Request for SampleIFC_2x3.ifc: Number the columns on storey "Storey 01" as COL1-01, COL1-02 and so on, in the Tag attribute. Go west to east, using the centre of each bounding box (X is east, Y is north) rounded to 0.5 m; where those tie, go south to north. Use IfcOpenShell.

First a look at what the model holds.

```python
import ifcopenshell
import ifcopenshell.util.element
import ifcopenshell.util.placement

model = ifcopenshell.open("SampleIFC_2x3.ifc")
print(model.schema)
storey = next(s for s in model.by_type("IfcBuildingStorey") if s.Name == "Storey 01")
columns = [e for e in ifcopenshell.util.element.get_decomposition(storey) if e.is_a("IfcColumn")]
for e in sorted(columns, key=lambda e: e.id()):
    origin = ifcopenshell.util.placement.get_local_placement(e.ObjectPlacement)[:3, 3]
    print(e.id(), e.Tag, e.Name, origin.round(2) + 0.0, sep=" | ")
```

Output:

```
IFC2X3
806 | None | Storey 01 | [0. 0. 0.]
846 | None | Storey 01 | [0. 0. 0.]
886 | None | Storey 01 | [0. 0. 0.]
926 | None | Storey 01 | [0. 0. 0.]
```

```python
import ifcopenshell
import ifcopenshell.geom
import ifcopenshell.util.element
import ifcopenshell.util.shape

model = ifcopenshell.open("SampleIFC_2x3.ifc")
settings = ifcopenshell.geom.settings()
settings.set("use-world-coords", True)


def centre(element):
    shape = ifcopenshell.geom.create_shape(settings, element)
    return ifcopenshell.util.shape.get_bbox_centroid(shape.geometry)


storey = next(s for s in model.by_type("IfcBuildingStorey") if s.Name == "Storey 01")
columns = [e for e in ifcopenshell.util.element.get_decomposition(storey) if e.is_a("IfcColumn")]

# Insertion points can sit at a corner or the storey origin, so sort by the geometry (in metres).
centres = {e: centre(e) for e in columns}
columns.sort(key=lambda e: (round(centres[e][0] / 0.5), centres[e][1]))

for i, e in enumerate(columns, start=1):
    number = f"COL1-{i:02d}"
    e.Tag = number
    print(e.id(), number)

model.write("SampleIFC_2x3_rev.ifc")
```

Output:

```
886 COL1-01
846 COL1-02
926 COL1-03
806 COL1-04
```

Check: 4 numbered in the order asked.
